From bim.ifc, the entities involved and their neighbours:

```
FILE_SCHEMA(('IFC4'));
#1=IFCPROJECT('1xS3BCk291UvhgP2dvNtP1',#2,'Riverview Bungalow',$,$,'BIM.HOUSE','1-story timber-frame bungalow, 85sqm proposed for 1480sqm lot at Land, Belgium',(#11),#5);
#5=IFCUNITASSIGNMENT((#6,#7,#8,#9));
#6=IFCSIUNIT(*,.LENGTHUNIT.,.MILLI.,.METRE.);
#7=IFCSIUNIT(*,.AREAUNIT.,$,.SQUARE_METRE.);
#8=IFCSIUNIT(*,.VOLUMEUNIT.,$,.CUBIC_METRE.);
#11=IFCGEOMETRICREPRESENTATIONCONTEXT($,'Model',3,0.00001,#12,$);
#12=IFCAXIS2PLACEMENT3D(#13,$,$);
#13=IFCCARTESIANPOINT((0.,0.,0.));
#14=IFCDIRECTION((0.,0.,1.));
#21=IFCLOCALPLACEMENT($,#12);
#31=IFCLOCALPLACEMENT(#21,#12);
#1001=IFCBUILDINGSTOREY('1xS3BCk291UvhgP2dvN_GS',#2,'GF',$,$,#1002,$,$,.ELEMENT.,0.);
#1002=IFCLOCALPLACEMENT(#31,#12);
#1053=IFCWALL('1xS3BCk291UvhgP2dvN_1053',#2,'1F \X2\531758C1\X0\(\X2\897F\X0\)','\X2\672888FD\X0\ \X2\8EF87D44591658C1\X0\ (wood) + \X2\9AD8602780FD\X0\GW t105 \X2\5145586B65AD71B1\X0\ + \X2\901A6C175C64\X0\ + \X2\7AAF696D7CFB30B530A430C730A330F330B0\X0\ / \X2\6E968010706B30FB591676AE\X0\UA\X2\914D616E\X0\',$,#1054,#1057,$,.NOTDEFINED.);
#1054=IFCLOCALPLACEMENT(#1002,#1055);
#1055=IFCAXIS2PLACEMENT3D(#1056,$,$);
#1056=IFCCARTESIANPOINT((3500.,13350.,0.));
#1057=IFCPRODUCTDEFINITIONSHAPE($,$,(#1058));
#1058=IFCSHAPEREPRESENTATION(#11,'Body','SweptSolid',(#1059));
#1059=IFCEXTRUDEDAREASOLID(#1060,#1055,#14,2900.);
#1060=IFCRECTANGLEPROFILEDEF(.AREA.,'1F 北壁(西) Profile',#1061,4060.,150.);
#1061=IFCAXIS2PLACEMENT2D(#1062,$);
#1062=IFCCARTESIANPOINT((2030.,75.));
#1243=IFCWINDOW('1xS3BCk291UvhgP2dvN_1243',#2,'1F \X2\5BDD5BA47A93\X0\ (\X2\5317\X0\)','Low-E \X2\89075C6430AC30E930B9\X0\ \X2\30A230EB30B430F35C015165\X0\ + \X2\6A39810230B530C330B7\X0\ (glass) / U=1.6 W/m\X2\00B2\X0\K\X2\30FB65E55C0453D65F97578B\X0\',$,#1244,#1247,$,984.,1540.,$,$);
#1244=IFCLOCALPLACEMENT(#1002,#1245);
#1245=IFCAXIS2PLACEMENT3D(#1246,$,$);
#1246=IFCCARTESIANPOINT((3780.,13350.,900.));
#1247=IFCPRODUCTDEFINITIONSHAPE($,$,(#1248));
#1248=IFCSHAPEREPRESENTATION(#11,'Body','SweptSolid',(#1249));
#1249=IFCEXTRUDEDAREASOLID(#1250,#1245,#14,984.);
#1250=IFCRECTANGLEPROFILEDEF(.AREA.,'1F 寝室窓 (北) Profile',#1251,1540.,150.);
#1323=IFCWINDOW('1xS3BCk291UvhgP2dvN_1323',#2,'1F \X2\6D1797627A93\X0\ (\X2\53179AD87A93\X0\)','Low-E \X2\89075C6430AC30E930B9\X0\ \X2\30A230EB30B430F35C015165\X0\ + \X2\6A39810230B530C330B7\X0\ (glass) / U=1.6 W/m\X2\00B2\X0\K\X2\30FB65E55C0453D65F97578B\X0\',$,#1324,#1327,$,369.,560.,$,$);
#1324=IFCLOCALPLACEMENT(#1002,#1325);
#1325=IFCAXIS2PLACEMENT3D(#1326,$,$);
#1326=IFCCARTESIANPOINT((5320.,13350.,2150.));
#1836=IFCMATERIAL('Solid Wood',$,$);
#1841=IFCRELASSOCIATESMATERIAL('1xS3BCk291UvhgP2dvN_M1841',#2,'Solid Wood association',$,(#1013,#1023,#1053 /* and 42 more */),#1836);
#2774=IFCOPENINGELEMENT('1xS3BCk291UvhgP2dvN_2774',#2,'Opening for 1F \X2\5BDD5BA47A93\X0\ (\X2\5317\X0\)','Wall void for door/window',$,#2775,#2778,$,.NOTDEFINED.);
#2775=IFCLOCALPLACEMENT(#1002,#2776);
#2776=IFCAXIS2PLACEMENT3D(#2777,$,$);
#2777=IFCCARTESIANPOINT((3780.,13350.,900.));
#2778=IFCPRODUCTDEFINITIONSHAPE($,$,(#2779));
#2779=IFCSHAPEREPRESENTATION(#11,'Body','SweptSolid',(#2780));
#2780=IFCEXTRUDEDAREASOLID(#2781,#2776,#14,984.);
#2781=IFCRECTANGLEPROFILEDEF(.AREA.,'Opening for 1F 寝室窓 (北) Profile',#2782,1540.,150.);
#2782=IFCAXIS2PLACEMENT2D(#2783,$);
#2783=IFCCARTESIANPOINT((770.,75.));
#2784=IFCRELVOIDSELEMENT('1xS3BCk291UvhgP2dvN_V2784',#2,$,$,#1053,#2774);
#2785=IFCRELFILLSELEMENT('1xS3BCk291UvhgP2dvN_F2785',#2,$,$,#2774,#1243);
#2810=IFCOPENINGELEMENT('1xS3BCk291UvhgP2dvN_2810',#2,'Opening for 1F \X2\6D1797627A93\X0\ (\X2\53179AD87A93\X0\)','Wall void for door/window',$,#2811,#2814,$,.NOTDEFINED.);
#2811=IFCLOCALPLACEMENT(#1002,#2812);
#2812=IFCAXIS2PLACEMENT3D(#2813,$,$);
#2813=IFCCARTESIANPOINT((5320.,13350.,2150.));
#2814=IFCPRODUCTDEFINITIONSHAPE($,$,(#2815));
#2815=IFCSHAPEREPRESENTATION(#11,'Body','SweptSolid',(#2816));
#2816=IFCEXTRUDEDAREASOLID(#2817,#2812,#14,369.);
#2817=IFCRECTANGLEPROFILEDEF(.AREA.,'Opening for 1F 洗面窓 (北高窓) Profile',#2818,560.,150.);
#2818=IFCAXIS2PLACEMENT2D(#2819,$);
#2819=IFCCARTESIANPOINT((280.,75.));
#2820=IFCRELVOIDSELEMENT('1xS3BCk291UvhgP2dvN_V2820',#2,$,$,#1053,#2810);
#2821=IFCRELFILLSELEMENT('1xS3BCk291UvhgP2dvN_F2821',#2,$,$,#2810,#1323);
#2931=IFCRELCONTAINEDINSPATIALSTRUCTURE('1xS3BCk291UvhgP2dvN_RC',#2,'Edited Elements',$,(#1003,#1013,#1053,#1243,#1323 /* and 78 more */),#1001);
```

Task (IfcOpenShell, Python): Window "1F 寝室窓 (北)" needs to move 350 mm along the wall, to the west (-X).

```python
import ifcopenshell
import ifcopenshell.api.geometry
import ifcopenshell.util.placement
import ifcopenshell.util.unit

model = ifcopenshell.open("bim.ifc")
unit_scale = ifcopenshell.util.unit.calculate_unit_scale(model)

window = model.by_guid("1xS3BCk291UvhgP2dvN_1243")
opening = window.FillsVoids[0].RelatingOpeningElement
wall = opening.VoidsElements[0].RelatingBuildingElement

wall_matrix = ifcopenshell.util.placement.get_local_placement(wall.ObjectPlacement)
shift = wall_matrix[:3, 0] * -0.35 / unit_scale
before = ifcopenshell.util.placement.get_local_placement(window.ObjectPlacement)[:3, 3].copy()

# The window is not placed relative to its opening, so move both.
for product in (opening, window):
    matrix = ifcopenshell.util.placement.get_local_placement(product.ObjectPlacement)
    matrix[:3, 3] += shift
    ifcopenshell.api.geometry.edit_object_placement(model, product=product, matrix=matrix, is_si=False)

after = ifcopenshell.util.placement.get_local_placement(window.ObjectPlacement)[:3, 3]
print("window moved by", (after - before).round(3) + 0.0)

model.write("bim_edited.ifc")
```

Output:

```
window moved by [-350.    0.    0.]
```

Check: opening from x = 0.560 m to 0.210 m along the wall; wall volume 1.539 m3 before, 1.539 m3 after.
